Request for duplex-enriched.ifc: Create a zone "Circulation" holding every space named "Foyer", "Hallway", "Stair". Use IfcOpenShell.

First a look at what the model holds.

```python
import ifcopenshell

model = ifcopenshell.open("duplex-enriched.ifc")
print(model.schema)
seen = {}
for space in model.by_type("IfcSpace"):
    seen[space.LongName] = seen.get(space.LongName, 0) + 1
for name, count in sorted(seen.items(), key=str):
    print(count, "x", name)
print("zones:", [z.Name for z in model.by_type("IfcZone")][:20])
```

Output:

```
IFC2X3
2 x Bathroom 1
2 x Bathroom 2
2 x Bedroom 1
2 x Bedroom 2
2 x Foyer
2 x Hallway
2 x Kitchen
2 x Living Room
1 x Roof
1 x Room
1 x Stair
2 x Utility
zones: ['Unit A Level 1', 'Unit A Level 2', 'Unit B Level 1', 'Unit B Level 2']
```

```python
import ifcopenshell
import ifcopenshell.api.group
import ifcopenshell.api.root

model = ifcopenshell.open("duplex-enriched.ifc")

names = {"Foyer", "Hallway", "Stair"}
spaces = [s for s in model.by_type("IfcSpace") if s.LongName in names]

zone = ifcopenshell.api.root.create_entity(model, ifc_class="IfcZone", name="Circulation")
ifcopenshell.api.group.assign_group(model, products=spaces, group=zone)
print(len(spaces), "spaces in", zone.Name)

model.write("duplex-enriched_updated.ifc")
```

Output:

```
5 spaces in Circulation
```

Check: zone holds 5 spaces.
